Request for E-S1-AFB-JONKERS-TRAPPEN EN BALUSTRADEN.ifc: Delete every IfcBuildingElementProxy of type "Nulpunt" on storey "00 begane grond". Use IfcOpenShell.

First a look at what the model holds.

```python
import ifcopenshell
import ifcopenshell.util.element

model = ifcopenshell.open("E-S1-AFB-JONKERS-TRAPPEN EN BALUSTRADEN.ifc")
print(model.schema)
storey = next(s for s in model.by_type("IfcBuildingStorey") if s.Name == "00 begane grond")
proxies = [e for e in ifcopenshell.util.element.get_decomposition(storey) if e.is_a("IfcBuildingElementProxy")]
seen = {}
for e in proxies:
    element_type = ifcopenshell.util.element.get_type(e)
    name = element_type.Name if element_type not in (None, e) else None
    seen[name] = seen.get(name, 0) + 1
for name, count in sorted(seen.items(), key=str):
    print(count, "x", name)
```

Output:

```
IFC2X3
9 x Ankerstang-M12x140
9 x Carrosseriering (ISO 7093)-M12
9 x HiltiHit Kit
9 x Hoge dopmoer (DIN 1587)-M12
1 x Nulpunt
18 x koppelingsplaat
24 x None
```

```python
import ifcopenshell
import ifcopenshell.api.root
import ifcopenshell.util.element

model = ifcopenshell.open("E-S1-AFB-JONKERS-TRAPPEN EN BALUSTRADEN.ifc")

storey = next(s for s in model.by_type("IfcBuildingStorey") if s.Name == "00 begane grond")
proxies = [e for e in ifcopenshell.util.element.get_decomposition(storey) if e.is_a("IfcBuildingElementProxy")]
targets = [e for e in proxies if (t := ifcopenshell.util.element.get_type(e)) not in (None, e) and t.Name == "Nulpunt"]

for e in targets:
    ifcopenshell.api.root.remove_product(model, product=e)
print(len(targets), "removed")

model.write("E-S1-AFB-JONKERS-TRAPPEN EN BALUSTRADEN_edited.ifc")
```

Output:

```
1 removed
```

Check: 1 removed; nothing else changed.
